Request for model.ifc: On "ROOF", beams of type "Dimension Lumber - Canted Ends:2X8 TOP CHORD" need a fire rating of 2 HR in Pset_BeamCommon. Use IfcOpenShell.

First a look at what the model holds.

```python
import ifcopenshell
import ifcopenshell.util.element

model = ifcopenshell.open("model.ifc")
print(model.schema)
storey = next(s for s in model.by_type("IfcBuildingStorey") if s.Name == "ROOF")
beams = [e for e in ifcopenshell.util.element.get_decomposition(storey) if e.is_a("IfcBeam")]
seen = {}
for e in beams:
    element_type = ifcopenshell.util.element.get_type(e)
    key = (element_type.Name if element_type != e and element_type else None, ifcopenshell.util.element.get_pset(e, "Pset_BeamCommon", "FireRating"))
    seen[key] = seen.get(key, 0) + 1
for (name, value), count in sorted(seen.items(), key=str):
    print(count, "x", name, "|", value)
```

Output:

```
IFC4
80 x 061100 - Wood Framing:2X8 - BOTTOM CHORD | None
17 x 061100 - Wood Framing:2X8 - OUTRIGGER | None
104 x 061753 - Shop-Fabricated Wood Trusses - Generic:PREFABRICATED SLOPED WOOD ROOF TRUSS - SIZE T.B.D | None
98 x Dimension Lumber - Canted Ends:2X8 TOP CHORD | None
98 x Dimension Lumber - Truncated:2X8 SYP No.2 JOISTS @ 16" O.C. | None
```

```python
import ifcopenshell
import ifcopenshell.api.pset
import ifcopenshell.util.element

model = ifcopenshell.open("model.ifc")

storey = next(s for s in model.by_type("IfcBuildingStorey") if s.Name == "ROOF")
beams = [e for e in ifcopenshell.util.element.get_decomposition(storey) if e.is_a("IfcBeam")]

count = 0
for e in beams:
    element_type = ifcopenshell.util.element.get_type(e)
    if element_type in (None, e) or element_type.Name != "Dimension Lumber - Canted Ends:2X8 TOP CHORD":
        continue
    # add_pset returns the element's existing set when there is one.
    pset = ifcopenshell.api.pset.add_pset(model, product=e, name="Pset_BeamCommon")
    ifcopenshell.api.pset.edit_pset(model, pset=pset, properties={"FireRating": "2 HR"})
    count += 1

print(count, "beams updated")

model.write("model_rev.ifc")
```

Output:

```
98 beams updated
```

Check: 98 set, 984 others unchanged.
